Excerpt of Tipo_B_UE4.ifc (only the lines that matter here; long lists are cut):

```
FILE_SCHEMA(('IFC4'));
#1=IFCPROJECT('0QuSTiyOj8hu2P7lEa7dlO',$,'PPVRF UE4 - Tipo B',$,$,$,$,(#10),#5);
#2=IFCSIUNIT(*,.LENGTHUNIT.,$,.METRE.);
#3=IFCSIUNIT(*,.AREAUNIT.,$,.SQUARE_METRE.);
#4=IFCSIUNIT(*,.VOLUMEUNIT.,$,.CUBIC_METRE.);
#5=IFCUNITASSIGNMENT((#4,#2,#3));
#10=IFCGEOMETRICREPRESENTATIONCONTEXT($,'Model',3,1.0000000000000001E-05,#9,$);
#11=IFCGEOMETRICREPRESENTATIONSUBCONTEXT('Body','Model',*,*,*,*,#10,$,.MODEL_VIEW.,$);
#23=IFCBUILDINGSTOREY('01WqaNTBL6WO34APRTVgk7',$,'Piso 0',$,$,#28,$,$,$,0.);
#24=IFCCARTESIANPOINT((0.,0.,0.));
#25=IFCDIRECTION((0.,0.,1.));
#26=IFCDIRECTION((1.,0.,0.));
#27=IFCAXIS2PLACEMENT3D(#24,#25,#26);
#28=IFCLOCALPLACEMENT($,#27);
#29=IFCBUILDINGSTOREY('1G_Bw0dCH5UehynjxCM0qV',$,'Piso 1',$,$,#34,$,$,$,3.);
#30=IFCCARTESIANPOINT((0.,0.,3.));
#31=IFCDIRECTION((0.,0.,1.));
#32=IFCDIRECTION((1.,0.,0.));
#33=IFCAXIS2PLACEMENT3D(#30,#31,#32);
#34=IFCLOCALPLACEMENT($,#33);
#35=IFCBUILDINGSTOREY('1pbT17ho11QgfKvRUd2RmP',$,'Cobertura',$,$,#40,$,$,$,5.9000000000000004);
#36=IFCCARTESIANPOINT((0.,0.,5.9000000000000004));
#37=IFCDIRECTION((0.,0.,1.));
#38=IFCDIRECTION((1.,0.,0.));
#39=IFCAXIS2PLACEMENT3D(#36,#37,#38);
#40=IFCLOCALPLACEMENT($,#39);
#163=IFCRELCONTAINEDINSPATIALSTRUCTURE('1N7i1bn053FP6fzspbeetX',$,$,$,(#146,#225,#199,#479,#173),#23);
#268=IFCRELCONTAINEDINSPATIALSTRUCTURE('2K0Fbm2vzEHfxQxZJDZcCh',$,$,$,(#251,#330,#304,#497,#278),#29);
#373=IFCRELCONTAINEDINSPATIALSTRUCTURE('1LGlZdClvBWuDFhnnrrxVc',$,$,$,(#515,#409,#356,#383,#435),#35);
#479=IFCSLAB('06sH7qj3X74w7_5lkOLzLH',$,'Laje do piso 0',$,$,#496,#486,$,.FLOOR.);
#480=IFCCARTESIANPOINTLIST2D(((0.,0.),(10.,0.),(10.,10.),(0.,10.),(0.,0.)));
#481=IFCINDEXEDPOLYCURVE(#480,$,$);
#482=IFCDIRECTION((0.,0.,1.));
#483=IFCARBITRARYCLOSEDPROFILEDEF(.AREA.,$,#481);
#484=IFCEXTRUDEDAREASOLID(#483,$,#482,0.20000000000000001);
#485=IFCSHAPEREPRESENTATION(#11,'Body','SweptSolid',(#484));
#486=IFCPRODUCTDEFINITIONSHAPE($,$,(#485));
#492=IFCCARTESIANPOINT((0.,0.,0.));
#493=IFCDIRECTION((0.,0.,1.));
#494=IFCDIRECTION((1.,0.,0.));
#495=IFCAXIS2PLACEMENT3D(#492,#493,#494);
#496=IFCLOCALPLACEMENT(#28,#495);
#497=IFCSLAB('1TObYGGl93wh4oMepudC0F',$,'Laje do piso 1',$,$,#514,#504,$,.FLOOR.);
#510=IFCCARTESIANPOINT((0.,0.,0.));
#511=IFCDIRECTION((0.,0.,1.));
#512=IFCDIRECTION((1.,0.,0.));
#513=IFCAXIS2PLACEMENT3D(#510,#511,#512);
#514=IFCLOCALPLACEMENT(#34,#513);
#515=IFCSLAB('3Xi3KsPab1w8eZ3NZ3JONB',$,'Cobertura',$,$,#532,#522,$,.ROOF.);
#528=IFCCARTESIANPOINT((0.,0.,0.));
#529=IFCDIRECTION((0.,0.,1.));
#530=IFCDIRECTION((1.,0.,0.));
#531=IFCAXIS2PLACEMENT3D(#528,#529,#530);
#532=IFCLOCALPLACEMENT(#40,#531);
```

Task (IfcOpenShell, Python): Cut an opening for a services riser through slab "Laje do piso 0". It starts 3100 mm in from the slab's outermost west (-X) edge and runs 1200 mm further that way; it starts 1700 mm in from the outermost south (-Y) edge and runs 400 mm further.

```python
import numpy as np
import ifcopenshell
import ifcopenshell.api.feature
import ifcopenshell.api.geometry
import ifcopenshell.api.root
import ifcopenshell.geom
import ifcopenshell.util.placement
import ifcopenshell.util.representation
import ifcopenshell.util.shape
import ifcopenshell.util.unit

model = ifcopenshell.open("Tipo_B_UE4.ifc")
unit_scale = ifcopenshell.util.unit.calculate_unit_scale(model)
settings = ifcopenshell.geom.settings()


def volume(element):
    """Net volume in cubic metres, openings subtracted."""
    shape = ifcopenshell.geom.create_shape(settings, element)
    return ifcopenshell.util.shape.get_volume(shape.geometry)


slab = model.by_guid("06sH7qj3X74w7_5lkOLzLH")
before = volume(slab)

# Extent in the slab's own axes, in metres. The edges named are its -X and -Y sides.
slab_shape = ifcopenshell.geom.create_shape(settings, slab)
vertices = ifcopenshell.util.shape.get_vertices(slab_shape.geometry)
x_min, y_min, bottom = vertices.min(axis=0)
top = vertices[:, 2].max()

opening = ifcopenshell.api.root.create_entity(model, ifc_class="IfcOpeningElement", name="Services riser opening", predefined_type="OPENING")
context = ifcopenshell.util.representation.get_context(model, "Model", "Body", "MODEL_VIEW")
width, depth = 1.2, 0.4
outline = [(0.0, 0.0), (width, 0.0), (width, depth), (0.0, depth), (0.0, 0.0)]
# Overshoot both faces by 50 mm so the cut is clean.
shape = ifcopenshell.api.geometry.add_slab_representation(
    model, context=context, depth=top - bottom + 0.1, polyline=outline
)
ifcopenshell.api.geometry.assign_representation(model, product=opening, representation=shape)

matrix = ifcopenshell.util.placement.get_local_placement(slab.ObjectPlacement)
matrix[:, 3] = matrix @ np.append(np.array([x_min + 3.1, y_min + 1.7, bottom - 0.05]) / unit_scale, 1.0)
ifcopenshell.api.geometry.edit_object_placement(model, product=opening, matrix=matrix, is_si=False)
ifcopenshell.api.feature.add_feature(model, feature=opening, element=slab)

after = volume(slab)

print(f"slab volume {before:.3f} -> {after:.3f} m3")

model.write("Tipo_B_UE4_rev.ifc")
```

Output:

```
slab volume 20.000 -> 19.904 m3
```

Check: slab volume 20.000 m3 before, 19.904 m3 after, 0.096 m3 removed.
